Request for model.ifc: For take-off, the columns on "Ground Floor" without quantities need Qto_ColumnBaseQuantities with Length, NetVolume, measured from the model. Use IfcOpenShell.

First a look at what the model holds.

```python
import ifcopenshell
import ifcopenshell.util.element
import ifcopenshell.util.unit

model = ifcopenshell.open("model.ifc")
print(model.schema)
for unit_type in ("LENGTHUNIT", "AREAUNIT", "VOLUMEUNIT"):
    print(unit_type, ifcopenshell.util.unit.calculate_unit_scale(model, unit_type))
storey = next(s for s in model.by_type("IfcBuildingStorey") if s.Name == "Ground Floor")
columns = [e for e in ifcopenshell.util.element.get_decomposition(storey) if e.is_a("IfcColumn")]
for e in sorted(columns, key=lambda e: e.id()):
    print(e.id(), e.is_a(), e.Name, list(ifcopenshell.util.element.get_psets(e, qtos_only=True)), sep=" | ")
```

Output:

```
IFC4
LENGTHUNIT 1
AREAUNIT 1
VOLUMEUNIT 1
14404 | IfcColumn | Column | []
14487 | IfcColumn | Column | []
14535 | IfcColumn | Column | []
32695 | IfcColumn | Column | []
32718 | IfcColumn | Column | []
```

```python
import ifcopenshell
import ifcopenshell.api.pset
import ifcopenshell.geom
import ifcopenshell.util.element
import ifcopenshell.util.shape
import ifcopenshell.util.unit

model = ifcopenshell.open("model.ifc")
unit_scale = ifcopenshell.util.unit.calculate_unit_scale(model)
volume_scale = ifcopenshell.util.unit.calculate_unit_scale(model, "VOLUMEUNIT")
settings = ifcopenshell.geom.settings()

storey = next(s for s in model.by_type("IfcBuildingStorey") if s.Name == "Ground Floor")
columns = [e for e in ifcopenshell.util.element.get_decomposition(storey) if e.is_a("IfcColumn")]

for e in sorted(columns, key=lambda e: e.id()):
    if ifcopenshell.util.element.get_psets(e, qtos_only=True, should_inherit=False):
        continue
    # Geometry comes back in metres, in the element's own axes.
    shape = ifcopenshell.geom.create_shape(settings, e)
    values = {
        "Length": ifcopenshell.util.shape.get_z(shape.geometry) / unit_scale,
        "NetVolume": ifcopenshell.util.shape.get_volume(shape.geometry) / volume_scale,
    }
    qto = ifcopenshell.api.pset.add_qto(model, product=e, name="Qto_ColumnBaseQuantities")
    ifcopenshell.api.pset.edit_qto(model, qto=qto, properties=values)
    print(e.id(), {k: round(v, 3) for k, v in values.items()})

model.write("model_v2.ifc")
```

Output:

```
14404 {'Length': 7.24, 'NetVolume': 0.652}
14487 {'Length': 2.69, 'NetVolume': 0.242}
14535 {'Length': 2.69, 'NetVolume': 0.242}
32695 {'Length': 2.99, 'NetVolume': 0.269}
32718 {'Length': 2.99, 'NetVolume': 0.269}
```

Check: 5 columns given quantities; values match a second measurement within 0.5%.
